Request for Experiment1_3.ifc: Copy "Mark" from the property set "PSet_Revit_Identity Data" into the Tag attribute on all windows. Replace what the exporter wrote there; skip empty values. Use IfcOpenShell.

First a look at what the model holds.

```python
import ifcopenshell
import ifcopenshell.util.element

model = ifcopenshell.open("Experiment1_3.ifc")
print(model.schema)
windows = model.by_type("IfcWindow")
print(len(windows), "windows")
for e in windows[:8]:
    source = ifcopenshell.util.element.get_pset(e, "PSet_Revit_Identity Data", "Mark")
    target = e.Tag
    print(e.id(), repr(source), repr(target), sep=" | ")
```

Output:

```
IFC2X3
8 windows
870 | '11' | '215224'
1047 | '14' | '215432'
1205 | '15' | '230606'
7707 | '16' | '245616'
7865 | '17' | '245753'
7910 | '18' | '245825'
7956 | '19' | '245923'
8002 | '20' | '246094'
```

```python
import ifcopenshell
import ifcopenshell.util.element

model = ifcopenshell.open("Experiment1_3.ifc")

count = 0
for e in model.by_type("IfcWindow"):
    value = ifcopenshell.util.element.get_pset(e, "PSet_Revit_Identity Data", "Mark")
    current = e.Tag
    if not value or not value.strip() or current == value:
        continue
    e.Tag = value
    count += 1

print(count, "windows updated")

model.write("Experiment1_3_edited.ifc")
```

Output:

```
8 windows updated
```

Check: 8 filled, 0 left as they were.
